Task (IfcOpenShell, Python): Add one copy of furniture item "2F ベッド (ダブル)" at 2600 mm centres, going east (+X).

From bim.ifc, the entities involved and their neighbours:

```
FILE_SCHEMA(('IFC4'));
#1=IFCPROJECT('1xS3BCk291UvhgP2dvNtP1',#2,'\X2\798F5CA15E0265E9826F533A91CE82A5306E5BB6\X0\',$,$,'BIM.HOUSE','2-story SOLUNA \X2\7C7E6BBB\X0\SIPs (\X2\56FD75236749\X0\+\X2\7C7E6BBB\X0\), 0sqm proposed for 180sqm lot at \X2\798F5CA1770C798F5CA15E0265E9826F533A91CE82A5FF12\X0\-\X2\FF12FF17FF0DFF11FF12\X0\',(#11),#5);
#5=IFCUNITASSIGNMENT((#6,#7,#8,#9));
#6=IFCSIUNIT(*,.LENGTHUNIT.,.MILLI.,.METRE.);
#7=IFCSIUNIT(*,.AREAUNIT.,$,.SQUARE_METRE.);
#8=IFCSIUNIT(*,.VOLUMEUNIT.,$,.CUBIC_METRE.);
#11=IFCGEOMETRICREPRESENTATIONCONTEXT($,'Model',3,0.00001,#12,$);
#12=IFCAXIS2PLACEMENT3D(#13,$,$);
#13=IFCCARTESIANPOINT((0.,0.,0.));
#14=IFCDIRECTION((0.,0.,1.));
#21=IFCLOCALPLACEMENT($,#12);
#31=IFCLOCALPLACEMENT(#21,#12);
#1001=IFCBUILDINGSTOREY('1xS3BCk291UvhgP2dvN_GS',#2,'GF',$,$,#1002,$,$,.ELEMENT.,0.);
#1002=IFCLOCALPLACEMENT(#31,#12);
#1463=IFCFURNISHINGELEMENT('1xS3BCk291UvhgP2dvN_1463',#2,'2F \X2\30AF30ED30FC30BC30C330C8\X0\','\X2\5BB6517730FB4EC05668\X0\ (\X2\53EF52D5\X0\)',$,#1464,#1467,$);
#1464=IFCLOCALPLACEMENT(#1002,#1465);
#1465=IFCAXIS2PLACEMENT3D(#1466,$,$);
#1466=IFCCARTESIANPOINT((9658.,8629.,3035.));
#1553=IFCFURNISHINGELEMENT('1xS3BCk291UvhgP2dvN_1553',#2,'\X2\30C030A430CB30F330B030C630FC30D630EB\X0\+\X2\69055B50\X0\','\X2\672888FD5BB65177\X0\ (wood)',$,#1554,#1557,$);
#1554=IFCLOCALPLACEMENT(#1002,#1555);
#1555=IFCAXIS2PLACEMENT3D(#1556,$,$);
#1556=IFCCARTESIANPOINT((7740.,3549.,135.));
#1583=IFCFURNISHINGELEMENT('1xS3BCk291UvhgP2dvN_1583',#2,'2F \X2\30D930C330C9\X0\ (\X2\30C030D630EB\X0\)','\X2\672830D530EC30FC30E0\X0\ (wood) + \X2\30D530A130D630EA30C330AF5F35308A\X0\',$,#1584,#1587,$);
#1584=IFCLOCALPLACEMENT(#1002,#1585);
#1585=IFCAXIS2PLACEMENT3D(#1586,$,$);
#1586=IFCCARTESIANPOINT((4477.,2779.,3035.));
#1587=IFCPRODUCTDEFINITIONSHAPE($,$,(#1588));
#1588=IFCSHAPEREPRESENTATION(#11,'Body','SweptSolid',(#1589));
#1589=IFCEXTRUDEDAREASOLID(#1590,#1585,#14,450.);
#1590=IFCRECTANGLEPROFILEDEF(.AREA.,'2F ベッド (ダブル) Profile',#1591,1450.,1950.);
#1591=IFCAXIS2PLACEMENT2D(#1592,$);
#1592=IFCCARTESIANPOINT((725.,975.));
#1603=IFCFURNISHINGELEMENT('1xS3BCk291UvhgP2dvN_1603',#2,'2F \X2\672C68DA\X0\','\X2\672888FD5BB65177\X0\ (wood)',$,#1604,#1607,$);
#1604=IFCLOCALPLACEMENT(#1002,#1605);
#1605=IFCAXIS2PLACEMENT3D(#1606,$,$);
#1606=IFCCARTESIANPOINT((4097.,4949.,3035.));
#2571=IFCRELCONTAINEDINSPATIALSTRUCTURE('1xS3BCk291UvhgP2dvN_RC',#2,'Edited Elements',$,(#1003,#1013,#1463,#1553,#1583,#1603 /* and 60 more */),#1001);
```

```python
import numpy as np
import ifcopenshell
import ifcopenshell.api.geometry
import ifcopenshell.api.root
import ifcopenshell.util.element
import ifcopenshell.util.placement

model = ifcopenshell.open("bim.ifc")


def reuse_history(source, copy):
    """copy_class also copies each property set's owner history, people and application; keep the originals."""
    for rel in copy.IsDefinedBy:
        if rel.is_a("IfcRelDefinesByProperties") and (history := rel.RelatingPropertyDefinition.OwnerHistory):
            rel.RelatingPropertyDefinition.OwnerHistory = source.OwnerHistory
            ifcopenshell.util.element.remove_deep2(model, history)


source = model.by_guid("1xS3BCk291UvhgP2dvN_1583")
base = ifcopenshell.util.placement.get_local_placement(source.ObjectPlacement)
step = np.array([1.0, 0.0, 0.0]) * 2600.0

for i in range(1, 2):
    copy = ifcopenshell.api.root.copy_class(model, product=source)
    copy.Representation = ifcopenshell.util.element.copy_deep(
        model, source.Representation, exclude=["IfcGeometricRepresentationContext", "IfcRepresentationMap"]
    )
    reuse_history(source, copy)
    matrix = base.copy()
    matrix[:3, 3] += i * step
    print("added at", matrix[:3, 3].round(3) + 0.0)
    ifcopenshell.api.geometry.edit_object_placement(model, product=copy, matrix=matrix, is_si=False)

model.write("bim-out.ifc")
```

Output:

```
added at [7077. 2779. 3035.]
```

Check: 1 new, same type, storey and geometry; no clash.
